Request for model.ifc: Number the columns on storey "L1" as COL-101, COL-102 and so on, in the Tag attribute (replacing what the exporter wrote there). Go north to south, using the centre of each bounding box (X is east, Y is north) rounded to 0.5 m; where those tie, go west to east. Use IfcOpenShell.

First a look at what the model holds.

```python
import ifcopenshell
import ifcopenshell.util.element
import ifcopenshell.util.placement

model = ifcopenshell.open("model.ifc")
print(model.schema)
storey = next(s for s in model.by_type("IfcBuildingStorey") if s.Name == "L1")
columns = [e for e in ifcopenshell.util.element.get_decomposition(storey) if e.is_a("IfcColumn")]
for e in sorted(columns, key=lambda e: e.id()):
    origin = ifcopenshell.util.placement.get_local_placement(e.ObjectPlacement)[:3, 3]
    print(e.id(), e.Tag, e.Name, origin.round(2) + 0.0, sep=" | ")
```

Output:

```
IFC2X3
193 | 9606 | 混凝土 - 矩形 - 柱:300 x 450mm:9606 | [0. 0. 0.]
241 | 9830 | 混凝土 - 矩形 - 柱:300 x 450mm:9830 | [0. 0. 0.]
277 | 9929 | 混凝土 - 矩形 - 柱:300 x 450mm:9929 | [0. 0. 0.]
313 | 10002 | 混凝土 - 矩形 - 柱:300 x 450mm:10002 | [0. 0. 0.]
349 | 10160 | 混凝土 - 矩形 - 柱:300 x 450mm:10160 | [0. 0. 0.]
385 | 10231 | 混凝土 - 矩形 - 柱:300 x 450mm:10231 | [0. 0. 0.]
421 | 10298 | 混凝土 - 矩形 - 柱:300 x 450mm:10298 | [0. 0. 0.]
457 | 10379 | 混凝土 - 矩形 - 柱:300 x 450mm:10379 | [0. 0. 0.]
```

```python
import ifcopenshell
import ifcopenshell.geom
import ifcopenshell.util.element
import ifcopenshell.util.shape

model = ifcopenshell.open("model.ifc")
settings = ifcopenshell.geom.settings()
settings.set("use-world-coords", True)


def centre(element):
    shape = ifcopenshell.geom.create_shape(settings, element)
    return ifcopenshell.util.shape.get_bbox_centroid(shape.geometry)


storey = next(s for s in model.by_type("IfcBuildingStorey") if s.Name == "L1")
columns = [e for e in ifcopenshell.util.element.get_decomposition(storey) if e.is_a("IfcColumn")]

# Insertion points can sit at a corner or the storey origin, so sort by the geometry (in metres).
centres = {e: centre(e) for e in columns}
columns.sort(key=lambda e: (-round(centres[e][1] / 0.5), centres[e][0]))

for i, e in enumerate(columns, start=1):
    number = f"COL-1{i:02d}"
    e.Tag = number
    print(e.id(), number)

model.write("model-out.ifc")
```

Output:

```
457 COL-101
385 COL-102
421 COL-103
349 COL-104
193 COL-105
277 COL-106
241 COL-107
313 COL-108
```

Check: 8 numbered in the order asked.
